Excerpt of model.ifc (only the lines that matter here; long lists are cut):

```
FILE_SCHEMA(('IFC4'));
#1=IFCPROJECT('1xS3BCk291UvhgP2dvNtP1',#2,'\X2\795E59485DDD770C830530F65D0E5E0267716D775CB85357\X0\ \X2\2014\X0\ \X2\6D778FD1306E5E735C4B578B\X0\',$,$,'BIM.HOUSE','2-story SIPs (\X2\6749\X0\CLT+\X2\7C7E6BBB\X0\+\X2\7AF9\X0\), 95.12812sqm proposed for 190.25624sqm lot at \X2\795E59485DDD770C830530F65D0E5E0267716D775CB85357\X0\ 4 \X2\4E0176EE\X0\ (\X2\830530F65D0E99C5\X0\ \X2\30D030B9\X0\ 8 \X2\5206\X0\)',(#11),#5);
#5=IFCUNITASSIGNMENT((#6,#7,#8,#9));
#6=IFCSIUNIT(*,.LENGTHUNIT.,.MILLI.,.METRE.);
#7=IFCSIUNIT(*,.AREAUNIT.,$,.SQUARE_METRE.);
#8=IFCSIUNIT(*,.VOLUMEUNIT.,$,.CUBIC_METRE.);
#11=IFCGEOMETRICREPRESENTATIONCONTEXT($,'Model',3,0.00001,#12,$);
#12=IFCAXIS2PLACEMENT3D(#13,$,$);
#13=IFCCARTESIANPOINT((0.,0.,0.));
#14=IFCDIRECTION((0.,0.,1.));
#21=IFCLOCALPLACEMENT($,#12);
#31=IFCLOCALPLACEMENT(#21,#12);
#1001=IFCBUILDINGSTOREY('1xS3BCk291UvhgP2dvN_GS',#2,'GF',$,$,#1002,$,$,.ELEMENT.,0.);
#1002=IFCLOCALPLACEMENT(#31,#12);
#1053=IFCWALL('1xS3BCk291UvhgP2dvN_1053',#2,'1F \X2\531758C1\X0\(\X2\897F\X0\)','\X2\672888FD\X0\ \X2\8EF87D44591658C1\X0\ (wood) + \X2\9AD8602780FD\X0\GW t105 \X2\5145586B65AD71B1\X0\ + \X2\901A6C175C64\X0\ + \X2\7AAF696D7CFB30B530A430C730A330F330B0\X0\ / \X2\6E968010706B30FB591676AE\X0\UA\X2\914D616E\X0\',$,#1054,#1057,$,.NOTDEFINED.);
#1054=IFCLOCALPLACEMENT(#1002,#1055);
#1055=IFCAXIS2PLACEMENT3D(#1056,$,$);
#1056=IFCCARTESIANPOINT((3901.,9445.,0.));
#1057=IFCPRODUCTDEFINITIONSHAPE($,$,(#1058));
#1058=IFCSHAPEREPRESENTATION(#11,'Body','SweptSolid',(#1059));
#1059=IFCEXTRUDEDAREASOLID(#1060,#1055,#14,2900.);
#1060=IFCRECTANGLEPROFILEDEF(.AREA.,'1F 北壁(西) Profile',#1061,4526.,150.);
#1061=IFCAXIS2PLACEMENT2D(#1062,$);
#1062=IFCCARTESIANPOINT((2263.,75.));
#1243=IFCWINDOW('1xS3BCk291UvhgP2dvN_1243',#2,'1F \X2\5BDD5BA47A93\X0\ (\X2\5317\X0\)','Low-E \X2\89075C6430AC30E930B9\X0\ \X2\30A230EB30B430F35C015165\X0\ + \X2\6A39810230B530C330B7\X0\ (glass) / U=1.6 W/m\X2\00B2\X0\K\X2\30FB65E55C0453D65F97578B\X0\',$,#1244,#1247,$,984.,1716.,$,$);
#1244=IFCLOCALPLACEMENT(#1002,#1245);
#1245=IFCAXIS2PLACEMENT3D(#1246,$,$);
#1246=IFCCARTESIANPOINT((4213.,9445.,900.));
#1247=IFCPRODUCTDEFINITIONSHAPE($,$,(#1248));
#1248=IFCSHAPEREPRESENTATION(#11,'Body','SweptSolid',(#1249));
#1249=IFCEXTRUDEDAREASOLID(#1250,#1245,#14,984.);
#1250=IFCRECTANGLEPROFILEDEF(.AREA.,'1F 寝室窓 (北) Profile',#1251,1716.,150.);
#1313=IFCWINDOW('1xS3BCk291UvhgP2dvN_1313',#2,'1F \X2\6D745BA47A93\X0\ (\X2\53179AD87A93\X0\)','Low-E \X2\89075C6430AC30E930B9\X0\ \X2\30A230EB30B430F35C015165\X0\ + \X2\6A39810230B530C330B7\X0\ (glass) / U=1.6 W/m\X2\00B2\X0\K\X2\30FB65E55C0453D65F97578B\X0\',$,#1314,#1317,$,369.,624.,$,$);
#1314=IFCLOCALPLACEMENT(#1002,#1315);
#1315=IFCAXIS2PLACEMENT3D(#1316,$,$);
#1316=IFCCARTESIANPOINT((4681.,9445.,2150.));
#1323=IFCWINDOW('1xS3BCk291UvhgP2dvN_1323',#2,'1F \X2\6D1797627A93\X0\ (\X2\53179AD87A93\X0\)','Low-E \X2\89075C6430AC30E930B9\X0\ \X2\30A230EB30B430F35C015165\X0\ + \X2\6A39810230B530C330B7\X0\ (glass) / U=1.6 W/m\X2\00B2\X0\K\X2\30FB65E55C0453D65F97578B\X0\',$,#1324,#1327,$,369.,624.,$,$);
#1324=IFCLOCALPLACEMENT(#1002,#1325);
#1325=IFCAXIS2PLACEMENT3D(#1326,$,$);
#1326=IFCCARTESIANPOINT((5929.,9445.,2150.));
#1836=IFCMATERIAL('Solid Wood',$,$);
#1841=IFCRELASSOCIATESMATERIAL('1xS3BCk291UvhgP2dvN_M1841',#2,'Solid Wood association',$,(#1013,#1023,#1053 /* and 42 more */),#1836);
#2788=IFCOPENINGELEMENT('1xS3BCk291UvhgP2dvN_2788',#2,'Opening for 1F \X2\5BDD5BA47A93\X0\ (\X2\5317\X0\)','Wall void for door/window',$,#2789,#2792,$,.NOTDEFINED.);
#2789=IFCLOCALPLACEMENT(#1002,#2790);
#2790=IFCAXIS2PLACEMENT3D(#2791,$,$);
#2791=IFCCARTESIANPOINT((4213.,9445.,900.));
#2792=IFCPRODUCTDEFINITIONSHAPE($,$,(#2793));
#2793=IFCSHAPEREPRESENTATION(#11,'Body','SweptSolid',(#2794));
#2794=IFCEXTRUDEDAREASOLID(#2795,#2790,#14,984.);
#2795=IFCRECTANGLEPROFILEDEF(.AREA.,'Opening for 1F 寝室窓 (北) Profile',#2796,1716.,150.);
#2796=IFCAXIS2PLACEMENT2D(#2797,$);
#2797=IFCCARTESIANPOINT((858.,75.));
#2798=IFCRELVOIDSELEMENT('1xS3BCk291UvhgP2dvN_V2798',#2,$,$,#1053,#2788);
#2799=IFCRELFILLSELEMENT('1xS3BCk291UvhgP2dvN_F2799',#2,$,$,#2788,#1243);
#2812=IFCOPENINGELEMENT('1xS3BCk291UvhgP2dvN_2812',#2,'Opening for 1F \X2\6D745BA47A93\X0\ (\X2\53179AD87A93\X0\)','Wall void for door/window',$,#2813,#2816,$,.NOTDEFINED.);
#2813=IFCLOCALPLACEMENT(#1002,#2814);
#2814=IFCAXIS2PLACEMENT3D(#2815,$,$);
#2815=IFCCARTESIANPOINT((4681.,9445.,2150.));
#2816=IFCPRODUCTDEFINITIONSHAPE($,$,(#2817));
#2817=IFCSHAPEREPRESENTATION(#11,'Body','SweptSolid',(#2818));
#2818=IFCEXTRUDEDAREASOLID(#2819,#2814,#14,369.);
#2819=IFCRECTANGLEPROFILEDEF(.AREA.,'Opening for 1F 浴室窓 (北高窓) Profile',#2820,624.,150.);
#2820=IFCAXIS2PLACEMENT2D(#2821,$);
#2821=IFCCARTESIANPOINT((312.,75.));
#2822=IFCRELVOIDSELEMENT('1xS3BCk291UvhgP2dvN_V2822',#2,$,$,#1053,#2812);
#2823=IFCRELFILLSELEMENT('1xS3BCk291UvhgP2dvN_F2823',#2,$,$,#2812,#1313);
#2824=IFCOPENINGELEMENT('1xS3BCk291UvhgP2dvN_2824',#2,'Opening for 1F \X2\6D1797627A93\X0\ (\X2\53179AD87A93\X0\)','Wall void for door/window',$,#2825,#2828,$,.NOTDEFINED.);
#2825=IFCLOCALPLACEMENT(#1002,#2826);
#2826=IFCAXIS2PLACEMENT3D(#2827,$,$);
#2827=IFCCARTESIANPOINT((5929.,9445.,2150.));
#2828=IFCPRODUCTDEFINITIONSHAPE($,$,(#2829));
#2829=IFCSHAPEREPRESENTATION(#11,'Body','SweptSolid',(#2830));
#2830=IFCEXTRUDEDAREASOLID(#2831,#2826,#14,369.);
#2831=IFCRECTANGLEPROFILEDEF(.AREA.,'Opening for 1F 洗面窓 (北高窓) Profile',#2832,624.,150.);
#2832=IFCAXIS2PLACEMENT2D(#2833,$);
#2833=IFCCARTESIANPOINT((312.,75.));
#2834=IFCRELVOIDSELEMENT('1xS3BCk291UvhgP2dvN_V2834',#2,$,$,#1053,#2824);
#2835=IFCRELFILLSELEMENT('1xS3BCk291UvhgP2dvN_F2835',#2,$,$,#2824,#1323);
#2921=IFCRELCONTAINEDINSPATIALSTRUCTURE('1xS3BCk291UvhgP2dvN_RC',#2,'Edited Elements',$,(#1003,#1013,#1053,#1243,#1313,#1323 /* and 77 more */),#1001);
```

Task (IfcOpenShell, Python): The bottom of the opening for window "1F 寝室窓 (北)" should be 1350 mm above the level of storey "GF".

```python
import numpy as np
import ifcopenshell
import ifcopenshell.api.geometry
import ifcopenshell.geom
import ifcopenshell.util.element
import ifcopenshell.util.placement
import ifcopenshell.util.shape
import ifcopenshell.util.unit

model = ifcopenshell.open("model.ifc")
unit_scale = ifcopenshell.util.unit.calculate_unit_scale(model)

window = model.by_guid("1xS3BCk291UvhgP2dvN_1243")
opening = window.FillsVoids[0].RelatingOpeningElement
storey = ifcopenshell.util.element.get_container(window, ifc_class="IfcBuildingStorey")
level = ifcopenshell.util.placement.get_local_placement(storey.ObjectPlacement)[2, 3]

# The opening's origin need not be at the sill, so measure its lowest point.
shape = ifcopenshell.geom.create_shape(ifcopenshell.geom.settings(), opening)
bottom = ifcopenshell.util.shape.get_shape_bottom_elevation(shape, shape.geometry) / unit_scale
dz = level + 1.35 / unit_scale - bottom

shift = np.array([0.0, 0.0, dz])
# The window is not placed relative to its opening, so move both.
for product in (opening, window):
    matrix = ifcopenshell.util.placement.get_local_placement(product.ObjectPlacement)
    matrix[:3, 3] += shift
    ifcopenshell.api.geometry.edit_object_placement(model, product=product, matrix=matrix, is_si=False)

print(f"moved by {dz * unit_scale:+.3f} m")

model.write("model_v2.ifc")
```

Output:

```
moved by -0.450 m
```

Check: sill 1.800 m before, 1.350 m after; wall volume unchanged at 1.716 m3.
